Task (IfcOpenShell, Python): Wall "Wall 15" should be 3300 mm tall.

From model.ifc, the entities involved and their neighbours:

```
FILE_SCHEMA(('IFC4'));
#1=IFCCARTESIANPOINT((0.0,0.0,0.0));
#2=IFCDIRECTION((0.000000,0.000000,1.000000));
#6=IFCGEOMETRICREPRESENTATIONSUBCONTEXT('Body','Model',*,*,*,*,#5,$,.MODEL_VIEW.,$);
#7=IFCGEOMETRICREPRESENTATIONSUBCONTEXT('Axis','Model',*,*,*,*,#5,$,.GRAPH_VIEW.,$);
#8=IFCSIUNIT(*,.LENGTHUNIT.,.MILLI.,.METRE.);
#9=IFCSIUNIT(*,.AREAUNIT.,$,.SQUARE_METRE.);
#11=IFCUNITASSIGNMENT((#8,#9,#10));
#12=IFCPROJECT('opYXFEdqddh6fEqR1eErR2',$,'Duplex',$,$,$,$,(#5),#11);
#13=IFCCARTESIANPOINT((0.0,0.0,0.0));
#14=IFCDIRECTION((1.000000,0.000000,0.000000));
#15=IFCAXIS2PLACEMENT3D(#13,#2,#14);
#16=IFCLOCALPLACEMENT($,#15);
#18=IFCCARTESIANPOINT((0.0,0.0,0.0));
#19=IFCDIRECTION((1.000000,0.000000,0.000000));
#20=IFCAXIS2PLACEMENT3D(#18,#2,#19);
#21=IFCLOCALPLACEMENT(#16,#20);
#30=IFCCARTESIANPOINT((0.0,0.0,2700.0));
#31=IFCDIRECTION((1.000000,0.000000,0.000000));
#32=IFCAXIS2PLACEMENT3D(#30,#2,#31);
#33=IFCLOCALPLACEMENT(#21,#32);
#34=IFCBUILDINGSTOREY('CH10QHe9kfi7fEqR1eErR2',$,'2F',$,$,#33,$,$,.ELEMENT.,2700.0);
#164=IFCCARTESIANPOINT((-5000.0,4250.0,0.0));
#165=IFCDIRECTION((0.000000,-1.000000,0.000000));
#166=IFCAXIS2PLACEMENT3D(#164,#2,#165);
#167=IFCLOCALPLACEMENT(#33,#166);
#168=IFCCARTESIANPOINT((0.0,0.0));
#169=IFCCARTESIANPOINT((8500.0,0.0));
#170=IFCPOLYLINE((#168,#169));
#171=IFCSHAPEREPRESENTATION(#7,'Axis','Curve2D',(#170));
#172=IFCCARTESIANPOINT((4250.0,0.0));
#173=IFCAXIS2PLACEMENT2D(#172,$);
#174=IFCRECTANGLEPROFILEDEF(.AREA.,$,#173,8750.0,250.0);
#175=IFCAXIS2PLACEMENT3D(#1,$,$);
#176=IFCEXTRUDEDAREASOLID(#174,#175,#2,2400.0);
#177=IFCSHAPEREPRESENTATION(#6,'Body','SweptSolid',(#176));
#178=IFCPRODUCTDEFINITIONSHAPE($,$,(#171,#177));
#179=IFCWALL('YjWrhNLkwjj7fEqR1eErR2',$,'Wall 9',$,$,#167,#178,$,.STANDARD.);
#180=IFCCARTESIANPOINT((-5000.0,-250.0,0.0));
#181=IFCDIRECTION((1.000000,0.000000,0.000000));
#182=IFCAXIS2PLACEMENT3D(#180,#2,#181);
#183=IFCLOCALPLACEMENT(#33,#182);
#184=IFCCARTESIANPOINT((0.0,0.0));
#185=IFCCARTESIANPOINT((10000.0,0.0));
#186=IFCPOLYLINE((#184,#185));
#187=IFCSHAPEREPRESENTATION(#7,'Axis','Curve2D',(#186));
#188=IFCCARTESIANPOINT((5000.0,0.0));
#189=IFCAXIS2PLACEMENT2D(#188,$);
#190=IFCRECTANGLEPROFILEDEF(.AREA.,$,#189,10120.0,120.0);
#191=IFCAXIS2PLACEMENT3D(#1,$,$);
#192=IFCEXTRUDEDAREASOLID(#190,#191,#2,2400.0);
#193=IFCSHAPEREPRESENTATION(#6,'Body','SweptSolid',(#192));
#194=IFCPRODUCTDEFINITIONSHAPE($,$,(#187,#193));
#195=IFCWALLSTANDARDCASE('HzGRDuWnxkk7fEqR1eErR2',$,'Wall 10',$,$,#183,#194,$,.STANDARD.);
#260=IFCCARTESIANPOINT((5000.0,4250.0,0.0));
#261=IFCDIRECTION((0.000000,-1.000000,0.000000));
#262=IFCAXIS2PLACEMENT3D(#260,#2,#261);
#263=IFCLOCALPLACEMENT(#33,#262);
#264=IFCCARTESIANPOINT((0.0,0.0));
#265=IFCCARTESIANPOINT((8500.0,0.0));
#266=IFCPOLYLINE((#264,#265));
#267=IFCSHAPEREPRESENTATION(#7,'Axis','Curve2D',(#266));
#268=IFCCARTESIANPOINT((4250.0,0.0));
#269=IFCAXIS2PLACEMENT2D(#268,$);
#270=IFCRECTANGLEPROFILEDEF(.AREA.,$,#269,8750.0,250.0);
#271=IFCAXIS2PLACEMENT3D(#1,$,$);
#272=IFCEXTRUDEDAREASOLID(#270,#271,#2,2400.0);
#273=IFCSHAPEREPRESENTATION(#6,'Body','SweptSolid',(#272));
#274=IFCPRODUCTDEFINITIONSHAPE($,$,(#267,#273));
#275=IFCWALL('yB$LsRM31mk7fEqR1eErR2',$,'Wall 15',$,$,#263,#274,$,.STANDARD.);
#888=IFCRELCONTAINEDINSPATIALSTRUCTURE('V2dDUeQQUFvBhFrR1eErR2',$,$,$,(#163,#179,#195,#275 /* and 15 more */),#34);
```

```python
import ifcopenshell
import ifcopenshell.geom
import ifcopenshell.util.representation
import ifcopenshell.util.shape
import ifcopenshell.util.unit

model = ifcopenshell.open("model.ifc")
unit_scale = ifcopenshell.util.unit.calculate_unit_scale(model)
settings = ifcopenshell.geom.settings()


def volume(element):
    """Net volume in cubic metres, openings subtracted."""
    shape = ifcopenshell.geom.create_shape(settings, element)
    return ifcopenshell.util.shape.get_volume(shape.geometry)


wall = model.by_guid("yB$LsRM31mk7fEqR1eErR2")
before = volume(wall)

body = ifcopenshell.util.representation.get_representation(wall, "Model", "Body")
solid = body.Items[0]
old_height = solid.Depth
solid.Depth = 3.3 / unit_scale
after = volume(wall)

print(f"height {old_height:g} -> {solid.Depth:g}, volume {before:.3f} -> {after:.3f} m3")

model.write("model_edited.ifc")
```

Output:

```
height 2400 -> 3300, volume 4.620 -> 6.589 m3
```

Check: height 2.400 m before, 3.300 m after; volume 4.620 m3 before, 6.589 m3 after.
